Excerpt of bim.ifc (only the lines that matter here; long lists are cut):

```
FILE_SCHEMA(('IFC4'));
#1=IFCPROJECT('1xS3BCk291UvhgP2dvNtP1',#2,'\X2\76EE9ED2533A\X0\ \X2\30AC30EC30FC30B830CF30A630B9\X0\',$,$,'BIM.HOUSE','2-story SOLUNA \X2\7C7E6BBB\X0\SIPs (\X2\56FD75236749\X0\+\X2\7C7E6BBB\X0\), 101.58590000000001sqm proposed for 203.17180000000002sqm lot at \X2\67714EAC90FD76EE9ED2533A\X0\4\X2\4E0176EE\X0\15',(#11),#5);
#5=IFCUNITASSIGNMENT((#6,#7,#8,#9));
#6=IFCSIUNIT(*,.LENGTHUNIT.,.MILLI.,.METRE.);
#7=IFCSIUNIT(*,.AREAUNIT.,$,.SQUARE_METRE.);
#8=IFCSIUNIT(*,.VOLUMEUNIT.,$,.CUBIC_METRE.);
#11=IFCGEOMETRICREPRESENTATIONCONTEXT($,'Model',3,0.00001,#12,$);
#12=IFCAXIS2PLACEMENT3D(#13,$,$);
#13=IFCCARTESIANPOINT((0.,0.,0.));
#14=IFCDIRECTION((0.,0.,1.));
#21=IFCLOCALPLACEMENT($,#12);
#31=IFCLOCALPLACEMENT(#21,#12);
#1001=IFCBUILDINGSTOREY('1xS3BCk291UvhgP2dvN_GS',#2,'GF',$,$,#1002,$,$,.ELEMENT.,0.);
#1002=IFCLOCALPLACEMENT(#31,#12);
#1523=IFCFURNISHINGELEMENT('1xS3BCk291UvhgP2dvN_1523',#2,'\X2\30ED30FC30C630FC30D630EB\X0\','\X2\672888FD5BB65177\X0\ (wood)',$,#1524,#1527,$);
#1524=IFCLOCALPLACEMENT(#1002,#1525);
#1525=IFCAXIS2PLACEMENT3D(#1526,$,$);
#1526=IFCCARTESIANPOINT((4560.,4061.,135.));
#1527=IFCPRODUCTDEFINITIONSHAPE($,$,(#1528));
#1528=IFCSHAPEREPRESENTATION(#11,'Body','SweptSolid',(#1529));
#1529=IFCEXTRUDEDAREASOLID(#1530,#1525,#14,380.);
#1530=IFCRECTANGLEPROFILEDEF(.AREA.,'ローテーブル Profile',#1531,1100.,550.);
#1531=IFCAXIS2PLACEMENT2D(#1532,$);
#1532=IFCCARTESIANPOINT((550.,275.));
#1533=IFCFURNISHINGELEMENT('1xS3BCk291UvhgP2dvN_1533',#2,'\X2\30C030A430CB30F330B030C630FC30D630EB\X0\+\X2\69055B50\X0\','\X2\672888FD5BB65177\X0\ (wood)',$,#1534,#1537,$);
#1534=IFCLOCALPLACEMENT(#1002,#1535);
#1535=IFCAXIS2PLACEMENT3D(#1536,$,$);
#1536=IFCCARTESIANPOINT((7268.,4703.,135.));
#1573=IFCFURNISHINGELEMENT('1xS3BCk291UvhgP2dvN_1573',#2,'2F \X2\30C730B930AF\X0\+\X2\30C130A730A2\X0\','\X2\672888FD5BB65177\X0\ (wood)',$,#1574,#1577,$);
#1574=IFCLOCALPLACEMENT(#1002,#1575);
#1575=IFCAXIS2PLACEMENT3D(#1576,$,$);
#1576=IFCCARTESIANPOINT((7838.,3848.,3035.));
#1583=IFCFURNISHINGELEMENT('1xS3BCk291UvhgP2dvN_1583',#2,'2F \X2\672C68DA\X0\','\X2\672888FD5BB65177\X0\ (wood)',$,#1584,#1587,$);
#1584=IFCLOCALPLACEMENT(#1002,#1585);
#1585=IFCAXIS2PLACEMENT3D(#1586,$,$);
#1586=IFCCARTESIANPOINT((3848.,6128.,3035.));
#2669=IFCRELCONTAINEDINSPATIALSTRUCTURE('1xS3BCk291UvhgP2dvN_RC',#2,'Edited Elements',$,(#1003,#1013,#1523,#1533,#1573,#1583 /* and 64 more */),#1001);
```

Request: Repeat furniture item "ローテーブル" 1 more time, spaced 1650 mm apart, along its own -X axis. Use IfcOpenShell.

```python
import ifcopenshell
import ifcopenshell.api.geometry
import ifcopenshell.api.root
import ifcopenshell.util.element
import ifcopenshell.util.placement
import ifcopenshell.util.unit

model = ifcopenshell.open("bim.ifc")
unit_scale = ifcopenshell.util.unit.calculate_unit_scale(model)


def reuse_history(source, copy):
    """copy_class also copies each property set's owner history, people and application; keep the originals."""
    for rel in copy.IsDefinedBy:
        if rel.is_a("IfcRelDefinesByProperties") and (history := rel.RelatingPropertyDefinition.OwnerHistory):
            rel.RelatingPropertyDefinition.OwnerHistory = source.OwnerHistory
            ifcopenshell.util.element.remove_deep2(model, history)


source = model.by_id(1523)
base = ifcopenshell.util.placement.get_local_placement(source.ObjectPlacement)
step = -base[:3, 0] * 1.65 / unit_scale

for i in range(1, 2):
    copy = ifcopenshell.api.root.copy_class(model, product=source)
    copy.Representation = ifcopenshell.util.element.copy_deep(
        model, source.Representation, exclude=["IfcGeometricRepresentationContext", "IfcRepresentationMap"]
    )
    reuse_history(source, copy)
    matrix = base.copy()
    matrix[:3, 3] += i * step
    print("added at", matrix[:3, 3].round(3) + 0.0)
    ifcopenshell.api.geometry.edit_object_placement(model, product=copy, matrix=matrix, is_si=False)

model.write("bim_rev.ifc")
```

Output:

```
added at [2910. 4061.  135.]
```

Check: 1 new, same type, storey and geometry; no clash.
